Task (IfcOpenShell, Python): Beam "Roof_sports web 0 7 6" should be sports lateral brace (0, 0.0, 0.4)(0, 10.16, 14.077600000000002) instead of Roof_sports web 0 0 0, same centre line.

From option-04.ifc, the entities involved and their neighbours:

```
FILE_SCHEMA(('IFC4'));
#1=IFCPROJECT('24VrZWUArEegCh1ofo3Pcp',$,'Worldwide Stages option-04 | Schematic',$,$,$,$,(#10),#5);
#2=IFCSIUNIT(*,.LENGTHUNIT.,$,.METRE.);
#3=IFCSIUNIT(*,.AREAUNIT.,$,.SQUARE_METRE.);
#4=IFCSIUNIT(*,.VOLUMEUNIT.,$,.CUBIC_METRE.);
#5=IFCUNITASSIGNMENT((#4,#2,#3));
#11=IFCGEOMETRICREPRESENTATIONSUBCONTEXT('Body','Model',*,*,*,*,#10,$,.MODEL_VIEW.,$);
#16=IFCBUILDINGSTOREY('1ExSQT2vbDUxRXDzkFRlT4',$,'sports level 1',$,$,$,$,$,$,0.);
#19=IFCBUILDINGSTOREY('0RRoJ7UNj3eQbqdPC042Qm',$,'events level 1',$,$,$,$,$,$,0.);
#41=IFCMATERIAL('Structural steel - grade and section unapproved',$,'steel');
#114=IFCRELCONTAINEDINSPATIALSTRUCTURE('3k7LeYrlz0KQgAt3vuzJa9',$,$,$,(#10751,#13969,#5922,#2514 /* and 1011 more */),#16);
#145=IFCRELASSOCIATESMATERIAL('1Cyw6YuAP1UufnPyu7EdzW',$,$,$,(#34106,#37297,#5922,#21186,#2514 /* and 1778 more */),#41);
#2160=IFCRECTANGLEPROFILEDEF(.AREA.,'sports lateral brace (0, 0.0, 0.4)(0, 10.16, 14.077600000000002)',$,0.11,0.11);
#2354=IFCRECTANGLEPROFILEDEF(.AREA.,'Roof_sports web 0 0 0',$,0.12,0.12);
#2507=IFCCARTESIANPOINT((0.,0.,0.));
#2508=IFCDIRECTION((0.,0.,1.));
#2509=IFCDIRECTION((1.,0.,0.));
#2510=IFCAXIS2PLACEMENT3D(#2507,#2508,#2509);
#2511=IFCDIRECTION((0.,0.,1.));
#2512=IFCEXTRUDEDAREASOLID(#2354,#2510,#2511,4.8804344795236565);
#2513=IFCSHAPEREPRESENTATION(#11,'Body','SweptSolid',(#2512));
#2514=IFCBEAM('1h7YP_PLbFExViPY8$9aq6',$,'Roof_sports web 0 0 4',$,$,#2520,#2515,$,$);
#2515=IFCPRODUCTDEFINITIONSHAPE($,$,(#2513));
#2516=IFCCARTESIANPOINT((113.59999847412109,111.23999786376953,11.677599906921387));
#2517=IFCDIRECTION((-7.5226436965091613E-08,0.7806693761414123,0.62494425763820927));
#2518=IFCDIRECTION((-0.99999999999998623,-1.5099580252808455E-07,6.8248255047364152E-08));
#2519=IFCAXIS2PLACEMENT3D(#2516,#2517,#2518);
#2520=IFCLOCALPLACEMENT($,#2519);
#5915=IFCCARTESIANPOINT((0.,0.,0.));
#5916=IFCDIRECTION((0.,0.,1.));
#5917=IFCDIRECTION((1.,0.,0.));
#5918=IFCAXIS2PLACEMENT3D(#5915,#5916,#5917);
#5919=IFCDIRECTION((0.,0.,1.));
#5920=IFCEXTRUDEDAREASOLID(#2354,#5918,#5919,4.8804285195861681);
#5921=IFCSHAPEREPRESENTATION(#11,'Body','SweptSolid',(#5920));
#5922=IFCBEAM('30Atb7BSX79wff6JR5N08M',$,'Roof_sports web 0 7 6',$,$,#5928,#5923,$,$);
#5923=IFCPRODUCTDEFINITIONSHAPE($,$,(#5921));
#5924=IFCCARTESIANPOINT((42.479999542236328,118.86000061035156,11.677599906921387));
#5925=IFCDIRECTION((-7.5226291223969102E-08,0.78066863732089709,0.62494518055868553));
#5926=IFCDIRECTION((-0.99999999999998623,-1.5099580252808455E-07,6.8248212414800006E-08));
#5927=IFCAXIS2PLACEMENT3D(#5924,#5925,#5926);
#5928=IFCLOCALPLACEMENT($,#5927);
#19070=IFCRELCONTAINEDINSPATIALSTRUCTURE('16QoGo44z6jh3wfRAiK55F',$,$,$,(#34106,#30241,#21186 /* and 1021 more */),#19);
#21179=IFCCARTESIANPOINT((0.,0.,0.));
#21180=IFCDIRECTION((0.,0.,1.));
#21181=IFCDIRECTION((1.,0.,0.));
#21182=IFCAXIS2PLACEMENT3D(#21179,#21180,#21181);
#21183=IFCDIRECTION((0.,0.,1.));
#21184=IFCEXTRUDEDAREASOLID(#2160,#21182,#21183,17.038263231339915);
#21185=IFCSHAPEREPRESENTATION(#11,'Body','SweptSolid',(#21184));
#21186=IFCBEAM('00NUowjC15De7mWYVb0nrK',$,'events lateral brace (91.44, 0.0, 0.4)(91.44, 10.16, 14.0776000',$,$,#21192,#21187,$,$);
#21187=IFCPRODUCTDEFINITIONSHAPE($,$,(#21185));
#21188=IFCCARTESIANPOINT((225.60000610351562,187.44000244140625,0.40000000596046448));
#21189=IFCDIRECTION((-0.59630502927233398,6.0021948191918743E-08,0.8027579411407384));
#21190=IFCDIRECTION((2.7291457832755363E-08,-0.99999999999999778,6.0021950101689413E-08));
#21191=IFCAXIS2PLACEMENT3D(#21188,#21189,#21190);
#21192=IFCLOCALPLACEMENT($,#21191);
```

```python
import ifcopenshell
import ifcopenshell.util.element
import ifcopenshell.util.representation

model = ifcopenshell.open("option-04.ifc")

member = model.by_guid("30Atb7BSX79wff6JR5N08M")
source = next(p for p in model.by_type("IfcRectangleProfileDef") if p.ProfileName == "sports lateral brace (0, 0.0, 0.4)(0, 10.16, 14.077600000000002)")

body = ifcopenshell.util.representation.get_representation(member, "Model", "Body")
solid = body.Items[0]
old_profile = solid.SweptArea

# Copy the section's sizes but keep this member's own profile position.
profile = ifcopenshell.util.element.copy(model, source)
profile.Position = old_profile.Position
solid.SweptArea = profile
if not model.get_total_inverses(old_profile):
    ifcopenshell.util.element.remove_deep2(model, old_profile)

print(solid.SweptArea)

model.write("option-04_rev.ifc")
```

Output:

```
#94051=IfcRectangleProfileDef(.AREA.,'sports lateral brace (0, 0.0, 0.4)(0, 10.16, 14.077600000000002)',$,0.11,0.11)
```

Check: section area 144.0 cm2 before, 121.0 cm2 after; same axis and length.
